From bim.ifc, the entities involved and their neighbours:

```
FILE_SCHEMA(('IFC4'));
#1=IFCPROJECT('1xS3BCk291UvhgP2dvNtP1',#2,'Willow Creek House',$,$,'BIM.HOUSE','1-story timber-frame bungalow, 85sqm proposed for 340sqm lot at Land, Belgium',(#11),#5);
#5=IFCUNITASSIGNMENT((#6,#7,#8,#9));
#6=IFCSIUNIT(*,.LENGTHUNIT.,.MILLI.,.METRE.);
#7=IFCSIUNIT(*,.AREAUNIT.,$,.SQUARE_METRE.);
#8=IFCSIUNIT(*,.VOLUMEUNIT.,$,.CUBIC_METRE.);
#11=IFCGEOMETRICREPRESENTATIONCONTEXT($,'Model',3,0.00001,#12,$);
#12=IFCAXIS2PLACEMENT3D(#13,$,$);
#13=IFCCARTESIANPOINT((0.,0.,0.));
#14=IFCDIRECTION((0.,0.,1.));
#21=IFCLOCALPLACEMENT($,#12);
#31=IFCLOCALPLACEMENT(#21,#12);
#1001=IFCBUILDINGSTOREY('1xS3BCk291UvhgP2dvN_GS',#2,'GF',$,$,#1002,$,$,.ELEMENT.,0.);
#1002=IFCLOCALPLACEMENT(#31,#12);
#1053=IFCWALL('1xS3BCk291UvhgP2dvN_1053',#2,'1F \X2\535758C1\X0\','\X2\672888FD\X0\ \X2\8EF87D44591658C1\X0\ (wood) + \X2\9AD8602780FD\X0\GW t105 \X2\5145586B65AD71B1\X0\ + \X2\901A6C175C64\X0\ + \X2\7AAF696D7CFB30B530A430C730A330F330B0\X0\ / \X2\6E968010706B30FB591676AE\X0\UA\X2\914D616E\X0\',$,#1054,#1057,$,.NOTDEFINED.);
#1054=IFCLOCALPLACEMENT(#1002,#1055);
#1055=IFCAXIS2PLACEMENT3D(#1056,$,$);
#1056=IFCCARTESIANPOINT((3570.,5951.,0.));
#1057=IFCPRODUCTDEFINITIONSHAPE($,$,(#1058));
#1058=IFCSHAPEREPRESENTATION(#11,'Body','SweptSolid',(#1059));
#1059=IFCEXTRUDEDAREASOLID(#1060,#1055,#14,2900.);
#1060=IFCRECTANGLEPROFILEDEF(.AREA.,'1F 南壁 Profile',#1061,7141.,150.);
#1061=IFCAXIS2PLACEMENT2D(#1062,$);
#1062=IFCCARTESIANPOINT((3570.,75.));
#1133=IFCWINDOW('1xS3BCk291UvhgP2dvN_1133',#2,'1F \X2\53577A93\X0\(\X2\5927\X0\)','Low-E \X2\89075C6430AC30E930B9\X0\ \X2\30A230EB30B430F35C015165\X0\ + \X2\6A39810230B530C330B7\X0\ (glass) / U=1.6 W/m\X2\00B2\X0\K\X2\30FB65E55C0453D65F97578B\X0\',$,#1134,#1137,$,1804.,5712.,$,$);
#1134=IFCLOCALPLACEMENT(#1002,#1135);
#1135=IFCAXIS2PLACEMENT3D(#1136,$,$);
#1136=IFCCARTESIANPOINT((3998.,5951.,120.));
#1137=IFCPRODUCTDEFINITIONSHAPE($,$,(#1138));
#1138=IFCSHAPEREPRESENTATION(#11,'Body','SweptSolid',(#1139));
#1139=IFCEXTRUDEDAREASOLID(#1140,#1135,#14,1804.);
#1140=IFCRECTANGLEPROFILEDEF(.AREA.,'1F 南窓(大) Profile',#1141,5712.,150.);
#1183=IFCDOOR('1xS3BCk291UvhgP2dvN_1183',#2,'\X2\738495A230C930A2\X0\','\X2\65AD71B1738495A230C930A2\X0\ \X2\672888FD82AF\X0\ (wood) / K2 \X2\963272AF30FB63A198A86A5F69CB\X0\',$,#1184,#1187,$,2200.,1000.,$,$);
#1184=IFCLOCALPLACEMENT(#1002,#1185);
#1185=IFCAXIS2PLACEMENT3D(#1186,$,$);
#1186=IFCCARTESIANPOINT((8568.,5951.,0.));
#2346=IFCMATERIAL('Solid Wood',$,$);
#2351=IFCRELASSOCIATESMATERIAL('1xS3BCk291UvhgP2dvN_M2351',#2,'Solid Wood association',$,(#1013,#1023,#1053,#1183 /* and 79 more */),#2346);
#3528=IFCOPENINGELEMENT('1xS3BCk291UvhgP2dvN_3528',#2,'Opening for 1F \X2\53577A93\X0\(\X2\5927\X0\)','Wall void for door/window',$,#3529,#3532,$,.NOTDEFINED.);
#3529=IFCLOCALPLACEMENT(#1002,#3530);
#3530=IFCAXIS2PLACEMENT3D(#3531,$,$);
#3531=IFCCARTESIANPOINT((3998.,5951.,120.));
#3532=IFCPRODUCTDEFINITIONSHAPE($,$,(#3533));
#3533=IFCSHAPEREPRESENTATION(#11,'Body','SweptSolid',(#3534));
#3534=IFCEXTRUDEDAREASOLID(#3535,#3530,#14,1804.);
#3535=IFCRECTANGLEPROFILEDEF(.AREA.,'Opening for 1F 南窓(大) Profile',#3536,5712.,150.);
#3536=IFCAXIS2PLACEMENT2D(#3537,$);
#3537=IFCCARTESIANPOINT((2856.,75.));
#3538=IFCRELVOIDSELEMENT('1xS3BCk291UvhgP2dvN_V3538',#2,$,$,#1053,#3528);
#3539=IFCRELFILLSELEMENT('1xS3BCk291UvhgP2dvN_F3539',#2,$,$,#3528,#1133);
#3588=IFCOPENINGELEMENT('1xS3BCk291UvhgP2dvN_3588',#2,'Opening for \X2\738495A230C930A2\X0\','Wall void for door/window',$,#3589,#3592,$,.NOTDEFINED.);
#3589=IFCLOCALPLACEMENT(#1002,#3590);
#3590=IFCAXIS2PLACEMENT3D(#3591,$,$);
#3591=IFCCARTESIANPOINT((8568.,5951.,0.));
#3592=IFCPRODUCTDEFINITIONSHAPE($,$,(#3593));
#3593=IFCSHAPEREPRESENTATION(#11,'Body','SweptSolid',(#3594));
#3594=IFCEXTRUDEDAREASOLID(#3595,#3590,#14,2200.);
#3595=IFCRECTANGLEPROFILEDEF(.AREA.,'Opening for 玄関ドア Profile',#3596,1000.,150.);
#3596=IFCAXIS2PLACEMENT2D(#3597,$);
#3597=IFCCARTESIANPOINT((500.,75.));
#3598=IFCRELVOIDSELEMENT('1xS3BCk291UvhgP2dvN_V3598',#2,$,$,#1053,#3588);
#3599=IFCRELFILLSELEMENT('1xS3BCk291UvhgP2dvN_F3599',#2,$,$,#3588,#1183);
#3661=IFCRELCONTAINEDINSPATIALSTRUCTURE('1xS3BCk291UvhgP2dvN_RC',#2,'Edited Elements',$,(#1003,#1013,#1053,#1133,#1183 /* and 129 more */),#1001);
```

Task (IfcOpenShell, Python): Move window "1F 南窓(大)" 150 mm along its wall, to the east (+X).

```python
import ifcopenshell
import ifcopenshell.api.geometry
import ifcopenshell.util.placement
import ifcopenshell.util.unit

model = ifcopenshell.open("bim.ifc")
unit_scale = ifcopenshell.util.unit.calculate_unit_scale(model)

window = model.by_guid("1xS3BCk291UvhgP2dvN_1133")
opening = window.FillsVoids[0].RelatingOpeningElement
wall = opening.VoidsElements[0].RelatingBuildingElement

wall_matrix = ifcopenshell.util.placement.get_local_placement(wall.ObjectPlacement)
shift = wall_matrix[:3, 0] * 0.15 / unit_scale
before = ifcopenshell.util.placement.get_local_placement(window.ObjectPlacement)[:3, 3].copy()

# The window is not placed relative to its opening, so move both.
for product in (opening, window):
    matrix = ifcopenshell.util.placement.get_local_placement(product.ObjectPlacement)
    matrix[:3, 3] += shift
    ifcopenshell.api.geometry.edit_object_placement(model, product=product, matrix=matrix, is_si=False)

after = ifcopenshell.util.placement.get_local_placement(window.ObjectPlacement)[:3, 3]
print("window moved by", (after - before).round(3) + 0.0)

model.write("bim_edited.ifc")
```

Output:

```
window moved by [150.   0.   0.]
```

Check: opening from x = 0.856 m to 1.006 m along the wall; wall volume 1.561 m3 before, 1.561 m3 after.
